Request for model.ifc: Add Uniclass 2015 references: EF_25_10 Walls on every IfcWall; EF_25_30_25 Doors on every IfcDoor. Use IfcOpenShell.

First a look at what the model holds.

```python
import ifcopenshell

model = ifcopenshell.open("model.ifc")
print(model.schema)
print("classifications:", [c.Name for c in model.by_type("IfcClassification")])
for ifc_class in ("IfcDoor", "IfcRoof", "IfcStair", "IfcWall", "IfcWindow"):
    print(ifc_class, len(model.by_type(ifc_class)))
```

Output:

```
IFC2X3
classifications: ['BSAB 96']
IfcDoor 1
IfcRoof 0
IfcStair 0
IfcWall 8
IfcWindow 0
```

```python
import ifcopenshell
import ifcopenshell.api.classification

model = ifcopenshell.open("model.ifc")

# IFC2X3 requires Source and Edition and has no link from the project to the system.
system = model.create_entity("IfcClassification", Source="NBS", Edition="2015", Name="Uniclass 2015")

codes = {
    "IfcWall": ("EF_25_10", "Walls"),
    "IfcDoor": ("EF_25_30_25", "Doors"),
}
for ifc_class, (code, name) in codes.items():
    products = model.by_type(ifc_class)
    ifcopenshell.api.classification.add_reference(
        model, products=products, classification=system, identification=code, name=name
    )
    print(code, len(products))

model.write("model_edited.ifc")
```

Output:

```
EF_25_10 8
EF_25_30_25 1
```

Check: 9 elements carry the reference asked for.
